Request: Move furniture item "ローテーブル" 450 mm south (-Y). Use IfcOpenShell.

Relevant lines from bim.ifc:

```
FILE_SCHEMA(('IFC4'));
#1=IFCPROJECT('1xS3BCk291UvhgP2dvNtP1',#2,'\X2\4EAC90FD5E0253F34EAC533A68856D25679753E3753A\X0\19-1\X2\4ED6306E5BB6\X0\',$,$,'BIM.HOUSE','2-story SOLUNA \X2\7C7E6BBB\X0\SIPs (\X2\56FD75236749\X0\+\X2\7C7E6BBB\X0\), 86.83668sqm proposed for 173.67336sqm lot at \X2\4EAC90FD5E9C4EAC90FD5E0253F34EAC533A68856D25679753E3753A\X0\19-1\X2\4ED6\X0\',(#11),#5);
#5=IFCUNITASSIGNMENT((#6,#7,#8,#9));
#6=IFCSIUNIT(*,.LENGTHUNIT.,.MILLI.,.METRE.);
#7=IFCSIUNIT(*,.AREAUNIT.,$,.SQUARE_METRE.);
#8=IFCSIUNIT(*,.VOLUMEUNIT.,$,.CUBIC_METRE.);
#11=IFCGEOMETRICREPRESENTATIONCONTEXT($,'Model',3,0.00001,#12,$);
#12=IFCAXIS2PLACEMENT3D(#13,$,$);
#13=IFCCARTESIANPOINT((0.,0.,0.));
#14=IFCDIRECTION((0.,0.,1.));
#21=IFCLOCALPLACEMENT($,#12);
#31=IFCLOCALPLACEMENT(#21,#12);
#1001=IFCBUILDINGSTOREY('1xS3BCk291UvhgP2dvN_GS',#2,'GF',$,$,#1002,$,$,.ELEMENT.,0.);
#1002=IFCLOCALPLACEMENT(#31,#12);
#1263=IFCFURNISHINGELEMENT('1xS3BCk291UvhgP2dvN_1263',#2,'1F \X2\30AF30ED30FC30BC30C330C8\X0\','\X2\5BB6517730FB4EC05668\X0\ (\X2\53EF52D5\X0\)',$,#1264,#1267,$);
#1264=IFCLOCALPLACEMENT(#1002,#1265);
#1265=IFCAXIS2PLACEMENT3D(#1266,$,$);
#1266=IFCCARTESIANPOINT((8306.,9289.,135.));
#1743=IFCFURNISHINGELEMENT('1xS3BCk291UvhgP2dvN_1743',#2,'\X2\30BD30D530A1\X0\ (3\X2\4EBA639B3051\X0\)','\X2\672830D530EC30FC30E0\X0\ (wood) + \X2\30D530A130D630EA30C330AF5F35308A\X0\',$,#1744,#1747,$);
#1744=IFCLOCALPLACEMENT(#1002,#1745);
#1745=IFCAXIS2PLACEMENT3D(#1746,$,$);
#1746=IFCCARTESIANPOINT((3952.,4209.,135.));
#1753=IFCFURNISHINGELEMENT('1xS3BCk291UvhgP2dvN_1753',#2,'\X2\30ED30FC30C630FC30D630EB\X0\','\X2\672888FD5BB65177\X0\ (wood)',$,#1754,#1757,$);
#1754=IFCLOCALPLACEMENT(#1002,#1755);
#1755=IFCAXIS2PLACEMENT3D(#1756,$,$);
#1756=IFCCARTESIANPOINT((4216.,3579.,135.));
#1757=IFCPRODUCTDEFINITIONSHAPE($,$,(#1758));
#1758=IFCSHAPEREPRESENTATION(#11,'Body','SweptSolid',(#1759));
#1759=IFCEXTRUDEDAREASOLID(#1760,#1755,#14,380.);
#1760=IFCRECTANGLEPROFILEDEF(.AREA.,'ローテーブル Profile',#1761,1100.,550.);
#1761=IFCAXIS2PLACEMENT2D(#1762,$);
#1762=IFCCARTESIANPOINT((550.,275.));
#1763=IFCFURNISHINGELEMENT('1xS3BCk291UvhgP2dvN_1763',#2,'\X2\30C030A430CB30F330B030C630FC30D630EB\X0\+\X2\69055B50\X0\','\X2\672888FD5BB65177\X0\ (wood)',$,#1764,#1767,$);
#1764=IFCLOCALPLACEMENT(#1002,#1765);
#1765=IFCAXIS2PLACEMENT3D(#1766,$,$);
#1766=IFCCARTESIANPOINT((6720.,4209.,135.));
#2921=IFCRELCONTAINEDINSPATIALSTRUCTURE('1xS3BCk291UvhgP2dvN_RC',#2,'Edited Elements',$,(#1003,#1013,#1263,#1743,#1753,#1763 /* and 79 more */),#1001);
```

```python
import ifcopenshell
import ifcopenshell.api.geometry
import ifcopenshell.util.placement

model = ifcopenshell.open("bim.ifc")

item = model.by_id(1753)
matrix = ifcopenshell.util.placement.get_local_placement(item.ObjectPlacement)
matrix[1, 3] -= 450.0
ifcopenshell.api.geometry.edit_object_placement(model, product=item, matrix=matrix, is_si=False)

print(ifcopenshell.util.placement.get_local_placement(item.ObjectPlacement).round(3) + 0.0)

model.write("bim-out.ifc")
```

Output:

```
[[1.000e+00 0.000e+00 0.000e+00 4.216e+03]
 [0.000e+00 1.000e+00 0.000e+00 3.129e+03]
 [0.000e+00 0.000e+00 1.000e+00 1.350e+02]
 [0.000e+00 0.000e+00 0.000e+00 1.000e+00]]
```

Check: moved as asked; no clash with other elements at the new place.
